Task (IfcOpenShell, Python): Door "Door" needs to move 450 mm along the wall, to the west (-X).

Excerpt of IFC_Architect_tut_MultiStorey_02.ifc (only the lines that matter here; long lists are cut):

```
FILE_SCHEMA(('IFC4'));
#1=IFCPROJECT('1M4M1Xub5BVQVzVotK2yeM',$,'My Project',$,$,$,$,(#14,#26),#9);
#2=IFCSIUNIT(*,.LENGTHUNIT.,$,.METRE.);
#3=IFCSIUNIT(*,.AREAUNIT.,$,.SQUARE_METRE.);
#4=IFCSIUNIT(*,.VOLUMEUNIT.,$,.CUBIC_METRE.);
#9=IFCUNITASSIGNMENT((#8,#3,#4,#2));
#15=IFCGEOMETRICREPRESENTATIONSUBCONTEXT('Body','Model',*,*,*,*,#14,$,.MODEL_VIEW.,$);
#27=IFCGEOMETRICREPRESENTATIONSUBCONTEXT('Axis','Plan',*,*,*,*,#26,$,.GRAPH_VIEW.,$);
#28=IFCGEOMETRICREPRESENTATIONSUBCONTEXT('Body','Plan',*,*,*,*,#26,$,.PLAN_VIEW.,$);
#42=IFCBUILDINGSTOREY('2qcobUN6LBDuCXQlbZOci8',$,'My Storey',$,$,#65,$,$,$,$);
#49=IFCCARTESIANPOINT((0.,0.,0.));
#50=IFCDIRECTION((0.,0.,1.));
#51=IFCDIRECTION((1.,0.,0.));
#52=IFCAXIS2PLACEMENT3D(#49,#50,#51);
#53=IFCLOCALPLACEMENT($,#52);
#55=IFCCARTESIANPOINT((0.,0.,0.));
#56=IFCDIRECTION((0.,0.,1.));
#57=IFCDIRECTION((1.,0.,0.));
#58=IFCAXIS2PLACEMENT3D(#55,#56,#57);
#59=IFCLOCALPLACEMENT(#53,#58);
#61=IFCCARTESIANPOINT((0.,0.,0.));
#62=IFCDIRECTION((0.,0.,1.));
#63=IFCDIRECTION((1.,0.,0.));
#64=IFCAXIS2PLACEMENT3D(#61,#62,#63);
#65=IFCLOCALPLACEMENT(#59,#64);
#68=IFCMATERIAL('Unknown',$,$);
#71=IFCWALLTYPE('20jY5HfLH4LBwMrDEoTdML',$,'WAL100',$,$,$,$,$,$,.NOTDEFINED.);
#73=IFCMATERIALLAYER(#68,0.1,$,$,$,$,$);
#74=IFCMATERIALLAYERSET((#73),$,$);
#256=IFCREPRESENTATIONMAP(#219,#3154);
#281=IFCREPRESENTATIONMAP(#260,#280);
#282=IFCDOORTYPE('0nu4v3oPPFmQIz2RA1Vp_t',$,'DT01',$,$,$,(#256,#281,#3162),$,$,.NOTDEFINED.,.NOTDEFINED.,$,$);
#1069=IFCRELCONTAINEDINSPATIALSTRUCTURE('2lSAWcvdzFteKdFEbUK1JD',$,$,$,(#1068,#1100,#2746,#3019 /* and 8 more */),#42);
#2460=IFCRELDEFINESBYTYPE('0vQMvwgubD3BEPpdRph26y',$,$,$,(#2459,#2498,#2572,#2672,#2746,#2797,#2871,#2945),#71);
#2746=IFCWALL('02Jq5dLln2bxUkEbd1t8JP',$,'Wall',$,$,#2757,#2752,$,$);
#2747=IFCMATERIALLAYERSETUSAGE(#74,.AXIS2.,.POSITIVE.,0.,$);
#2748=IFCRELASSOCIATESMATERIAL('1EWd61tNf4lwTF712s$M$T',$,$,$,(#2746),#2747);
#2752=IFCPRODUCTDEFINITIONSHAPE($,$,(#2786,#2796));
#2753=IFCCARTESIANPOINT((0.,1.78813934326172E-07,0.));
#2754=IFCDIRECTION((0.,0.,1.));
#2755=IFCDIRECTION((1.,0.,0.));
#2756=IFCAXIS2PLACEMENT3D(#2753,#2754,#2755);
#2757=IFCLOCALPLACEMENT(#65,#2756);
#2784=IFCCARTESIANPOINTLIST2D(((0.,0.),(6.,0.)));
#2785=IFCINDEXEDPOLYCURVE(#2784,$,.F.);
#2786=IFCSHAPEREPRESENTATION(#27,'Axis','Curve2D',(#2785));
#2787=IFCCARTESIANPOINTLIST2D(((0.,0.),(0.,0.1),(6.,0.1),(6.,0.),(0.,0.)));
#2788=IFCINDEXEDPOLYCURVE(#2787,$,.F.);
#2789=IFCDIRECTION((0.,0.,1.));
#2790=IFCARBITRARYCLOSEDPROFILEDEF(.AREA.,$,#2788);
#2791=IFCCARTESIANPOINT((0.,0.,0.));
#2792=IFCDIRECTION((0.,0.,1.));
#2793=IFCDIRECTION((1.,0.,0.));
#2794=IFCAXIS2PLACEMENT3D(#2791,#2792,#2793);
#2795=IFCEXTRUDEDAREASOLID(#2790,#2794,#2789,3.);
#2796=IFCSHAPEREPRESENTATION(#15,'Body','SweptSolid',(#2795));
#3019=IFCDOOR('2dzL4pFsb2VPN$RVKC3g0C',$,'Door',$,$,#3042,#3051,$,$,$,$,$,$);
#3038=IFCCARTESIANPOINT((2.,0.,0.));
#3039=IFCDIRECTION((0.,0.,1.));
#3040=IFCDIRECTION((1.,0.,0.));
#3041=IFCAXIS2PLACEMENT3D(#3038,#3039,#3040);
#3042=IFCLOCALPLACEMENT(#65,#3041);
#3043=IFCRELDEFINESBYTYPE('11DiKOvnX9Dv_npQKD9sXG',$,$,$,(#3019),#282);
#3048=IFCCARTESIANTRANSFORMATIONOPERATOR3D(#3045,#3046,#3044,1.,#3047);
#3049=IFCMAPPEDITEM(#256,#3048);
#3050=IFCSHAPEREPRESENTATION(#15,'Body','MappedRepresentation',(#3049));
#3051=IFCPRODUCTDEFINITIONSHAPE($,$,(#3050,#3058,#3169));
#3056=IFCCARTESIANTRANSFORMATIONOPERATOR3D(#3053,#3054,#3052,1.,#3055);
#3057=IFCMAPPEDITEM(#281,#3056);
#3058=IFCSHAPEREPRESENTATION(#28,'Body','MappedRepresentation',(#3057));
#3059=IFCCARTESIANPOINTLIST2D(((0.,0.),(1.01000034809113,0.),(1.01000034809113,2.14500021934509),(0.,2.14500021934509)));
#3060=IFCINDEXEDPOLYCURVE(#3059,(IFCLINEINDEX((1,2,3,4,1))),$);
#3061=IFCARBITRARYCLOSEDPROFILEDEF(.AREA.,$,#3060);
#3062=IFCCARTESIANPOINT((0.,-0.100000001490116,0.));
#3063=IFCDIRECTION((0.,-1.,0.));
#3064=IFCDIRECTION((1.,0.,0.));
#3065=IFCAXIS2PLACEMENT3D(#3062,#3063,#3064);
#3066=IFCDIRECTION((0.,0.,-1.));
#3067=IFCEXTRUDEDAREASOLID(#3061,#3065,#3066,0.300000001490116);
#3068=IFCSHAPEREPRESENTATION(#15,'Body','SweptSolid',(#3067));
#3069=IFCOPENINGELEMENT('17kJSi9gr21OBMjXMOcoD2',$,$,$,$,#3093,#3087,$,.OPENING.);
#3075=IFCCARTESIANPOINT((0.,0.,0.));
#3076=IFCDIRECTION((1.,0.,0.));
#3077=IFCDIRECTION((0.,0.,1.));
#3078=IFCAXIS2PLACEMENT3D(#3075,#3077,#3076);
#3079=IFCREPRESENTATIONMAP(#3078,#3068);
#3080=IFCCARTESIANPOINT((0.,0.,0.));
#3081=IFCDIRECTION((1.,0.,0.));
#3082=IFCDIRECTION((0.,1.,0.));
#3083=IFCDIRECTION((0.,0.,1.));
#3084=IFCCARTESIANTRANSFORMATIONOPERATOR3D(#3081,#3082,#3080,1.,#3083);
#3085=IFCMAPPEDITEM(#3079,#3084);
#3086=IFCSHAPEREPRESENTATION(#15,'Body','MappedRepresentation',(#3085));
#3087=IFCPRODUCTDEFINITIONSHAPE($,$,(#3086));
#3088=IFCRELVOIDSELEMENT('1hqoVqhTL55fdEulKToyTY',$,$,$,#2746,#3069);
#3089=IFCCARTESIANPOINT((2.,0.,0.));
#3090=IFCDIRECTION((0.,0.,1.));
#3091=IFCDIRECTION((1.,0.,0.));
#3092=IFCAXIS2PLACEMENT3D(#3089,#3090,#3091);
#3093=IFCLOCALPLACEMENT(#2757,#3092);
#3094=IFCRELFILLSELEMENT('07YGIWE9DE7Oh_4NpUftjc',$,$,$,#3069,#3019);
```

```python
import ifcopenshell
import ifcopenshell.api.geometry
import ifcopenshell.util.placement

model = ifcopenshell.open("IFC_Architect_tut_MultiStorey_02.ifc")

door = model.by_guid("2dzL4pFsb2VPN$RVKC3g0C")
opening = door.FillsVoids[0].RelatingOpeningElement
wall = opening.VoidsElements[0].RelatingBuildingElement

wall_matrix = ifcopenshell.util.placement.get_local_placement(wall.ObjectPlacement)
shift = wall_matrix[:3, 0] * -0.45
before = ifcopenshell.util.placement.get_local_placement(door.ObjectPlacement)[:3, 3].copy()

# The door is not placed relative to its opening, so move both.
for product in (opening, door):
    matrix = ifcopenshell.util.placement.get_local_placement(product.ObjectPlacement)
    matrix[:3, 3] += shift
    ifcopenshell.api.geometry.edit_object_placement(model, product=product, matrix=matrix, is_si=False)

after = ifcopenshell.util.placement.get_local_placement(door.ObjectPlacement)[:3, 3]
print("door moved by", (after - before).round(3) + 0.0)

model.write("IFC_Architect_tut_MultiStorey_02_updated.ifc")
```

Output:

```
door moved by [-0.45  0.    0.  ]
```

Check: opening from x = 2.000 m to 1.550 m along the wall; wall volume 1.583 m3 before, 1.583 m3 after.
